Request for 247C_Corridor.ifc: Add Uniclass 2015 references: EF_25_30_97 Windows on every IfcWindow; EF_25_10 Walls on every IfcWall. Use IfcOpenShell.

First a look at what the model holds.

```python
import ifcopenshell

model = ifcopenshell.open("247C_Corridor.ifc")
print(model.schema)
print("classifications:", [c.Name for c in model.by_type("IfcClassification")])
for ifc_class in ("IfcDoor", "IfcRoof", "IfcStair", "IfcWall", "IfcWindow"):
    print(ifc_class, len(model.by_type(ifc_class)))
```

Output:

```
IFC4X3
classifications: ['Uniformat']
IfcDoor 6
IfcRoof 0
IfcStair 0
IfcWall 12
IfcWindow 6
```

```python
import ifcopenshell
import ifcopenshell.api.classification

model = ifcopenshell.open("247C_Corridor.ifc")

system = ifcopenshell.api.classification.add_classification(model, classification="Uniclass 2015")

codes = {
    "IfcWindow": ("EF_25_30_97", "Windows"),
    "IfcWall": ("EF_25_10", "Walls"),
}
for ifc_class, (code, name) in codes.items():
    products = model.by_type(ifc_class)
    ifcopenshell.api.classification.add_reference(
        model, products=products, classification=system, identification=code, name=name
    )
    print(code, len(products))

model.write("247C_Corridor_rev.ifc")
```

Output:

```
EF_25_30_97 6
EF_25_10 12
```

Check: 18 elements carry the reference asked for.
